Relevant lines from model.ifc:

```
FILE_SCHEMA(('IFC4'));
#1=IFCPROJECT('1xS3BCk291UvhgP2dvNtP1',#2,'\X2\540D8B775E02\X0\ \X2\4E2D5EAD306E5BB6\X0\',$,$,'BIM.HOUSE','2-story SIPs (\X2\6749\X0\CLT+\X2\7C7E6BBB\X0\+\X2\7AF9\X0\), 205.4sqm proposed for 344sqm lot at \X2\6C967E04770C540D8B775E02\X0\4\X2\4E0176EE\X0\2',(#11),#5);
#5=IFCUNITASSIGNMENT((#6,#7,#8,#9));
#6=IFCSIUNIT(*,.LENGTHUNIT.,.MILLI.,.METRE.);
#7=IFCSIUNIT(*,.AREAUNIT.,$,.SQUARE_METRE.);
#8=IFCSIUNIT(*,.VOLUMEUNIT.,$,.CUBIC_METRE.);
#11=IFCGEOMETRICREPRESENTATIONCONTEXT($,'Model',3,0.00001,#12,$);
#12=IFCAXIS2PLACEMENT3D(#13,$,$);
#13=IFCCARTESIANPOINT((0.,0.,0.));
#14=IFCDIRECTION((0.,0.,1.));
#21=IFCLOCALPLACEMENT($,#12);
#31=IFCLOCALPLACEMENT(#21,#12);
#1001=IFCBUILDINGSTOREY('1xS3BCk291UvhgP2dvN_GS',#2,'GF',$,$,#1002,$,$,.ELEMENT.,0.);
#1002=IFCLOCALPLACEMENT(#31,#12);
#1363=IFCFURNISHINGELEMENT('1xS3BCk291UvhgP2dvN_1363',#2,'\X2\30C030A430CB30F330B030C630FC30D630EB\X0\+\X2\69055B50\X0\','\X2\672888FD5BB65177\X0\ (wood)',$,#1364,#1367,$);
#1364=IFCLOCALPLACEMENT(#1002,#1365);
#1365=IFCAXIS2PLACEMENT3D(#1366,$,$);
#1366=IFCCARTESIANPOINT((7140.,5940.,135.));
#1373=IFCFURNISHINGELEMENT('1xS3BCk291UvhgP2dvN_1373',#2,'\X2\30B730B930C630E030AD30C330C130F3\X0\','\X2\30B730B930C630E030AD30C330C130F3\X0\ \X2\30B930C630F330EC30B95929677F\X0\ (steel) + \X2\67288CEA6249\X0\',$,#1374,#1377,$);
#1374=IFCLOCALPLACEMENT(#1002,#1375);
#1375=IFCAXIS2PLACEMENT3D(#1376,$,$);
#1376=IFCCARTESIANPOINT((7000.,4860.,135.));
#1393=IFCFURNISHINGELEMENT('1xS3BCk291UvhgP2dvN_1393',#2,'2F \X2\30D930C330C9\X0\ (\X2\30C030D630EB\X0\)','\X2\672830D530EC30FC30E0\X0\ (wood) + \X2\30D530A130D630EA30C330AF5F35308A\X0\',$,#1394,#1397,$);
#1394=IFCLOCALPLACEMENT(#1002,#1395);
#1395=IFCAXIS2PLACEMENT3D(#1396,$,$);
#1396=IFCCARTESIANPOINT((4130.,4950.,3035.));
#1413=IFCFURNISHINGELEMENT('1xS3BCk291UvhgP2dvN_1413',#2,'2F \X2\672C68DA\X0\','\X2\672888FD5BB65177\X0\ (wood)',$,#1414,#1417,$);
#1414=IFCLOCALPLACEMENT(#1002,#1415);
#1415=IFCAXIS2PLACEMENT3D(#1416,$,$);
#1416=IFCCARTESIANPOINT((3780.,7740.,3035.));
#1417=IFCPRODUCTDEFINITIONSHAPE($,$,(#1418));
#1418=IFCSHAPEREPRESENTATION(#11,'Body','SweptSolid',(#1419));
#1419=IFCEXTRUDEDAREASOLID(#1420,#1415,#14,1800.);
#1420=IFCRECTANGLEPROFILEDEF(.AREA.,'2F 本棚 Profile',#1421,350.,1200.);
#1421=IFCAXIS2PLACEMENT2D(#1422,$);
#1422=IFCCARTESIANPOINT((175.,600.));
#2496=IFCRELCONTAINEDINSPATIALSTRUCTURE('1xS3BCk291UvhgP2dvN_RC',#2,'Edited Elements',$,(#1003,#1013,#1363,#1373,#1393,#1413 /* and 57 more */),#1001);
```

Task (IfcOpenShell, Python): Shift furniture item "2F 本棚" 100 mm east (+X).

```python
import ifcopenshell
import ifcopenshell.api.geometry
import ifcopenshell.util.placement

model = ifcopenshell.open("model.ifc")

item = model.by_guid("1xS3BCk291UvhgP2dvN_1413")
matrix = ifcopenshell.util.placement.get_local_placement(item.ObjectPlacement)
matrix[0, 3] += 100.0
ifcopenshell.api.geometry.edit_object_placement(model, product=item, matrix=matrix, is_si=False)

print(ifcopenshell.util.placement.get_local_placement(item.ObjectPlacement).round(3) + 0.0)

model.write("model-out.ifc")
```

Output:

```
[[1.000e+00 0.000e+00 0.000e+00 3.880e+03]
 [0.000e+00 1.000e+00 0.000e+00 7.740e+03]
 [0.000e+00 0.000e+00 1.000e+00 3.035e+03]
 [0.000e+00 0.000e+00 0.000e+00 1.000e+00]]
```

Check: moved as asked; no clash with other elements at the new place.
